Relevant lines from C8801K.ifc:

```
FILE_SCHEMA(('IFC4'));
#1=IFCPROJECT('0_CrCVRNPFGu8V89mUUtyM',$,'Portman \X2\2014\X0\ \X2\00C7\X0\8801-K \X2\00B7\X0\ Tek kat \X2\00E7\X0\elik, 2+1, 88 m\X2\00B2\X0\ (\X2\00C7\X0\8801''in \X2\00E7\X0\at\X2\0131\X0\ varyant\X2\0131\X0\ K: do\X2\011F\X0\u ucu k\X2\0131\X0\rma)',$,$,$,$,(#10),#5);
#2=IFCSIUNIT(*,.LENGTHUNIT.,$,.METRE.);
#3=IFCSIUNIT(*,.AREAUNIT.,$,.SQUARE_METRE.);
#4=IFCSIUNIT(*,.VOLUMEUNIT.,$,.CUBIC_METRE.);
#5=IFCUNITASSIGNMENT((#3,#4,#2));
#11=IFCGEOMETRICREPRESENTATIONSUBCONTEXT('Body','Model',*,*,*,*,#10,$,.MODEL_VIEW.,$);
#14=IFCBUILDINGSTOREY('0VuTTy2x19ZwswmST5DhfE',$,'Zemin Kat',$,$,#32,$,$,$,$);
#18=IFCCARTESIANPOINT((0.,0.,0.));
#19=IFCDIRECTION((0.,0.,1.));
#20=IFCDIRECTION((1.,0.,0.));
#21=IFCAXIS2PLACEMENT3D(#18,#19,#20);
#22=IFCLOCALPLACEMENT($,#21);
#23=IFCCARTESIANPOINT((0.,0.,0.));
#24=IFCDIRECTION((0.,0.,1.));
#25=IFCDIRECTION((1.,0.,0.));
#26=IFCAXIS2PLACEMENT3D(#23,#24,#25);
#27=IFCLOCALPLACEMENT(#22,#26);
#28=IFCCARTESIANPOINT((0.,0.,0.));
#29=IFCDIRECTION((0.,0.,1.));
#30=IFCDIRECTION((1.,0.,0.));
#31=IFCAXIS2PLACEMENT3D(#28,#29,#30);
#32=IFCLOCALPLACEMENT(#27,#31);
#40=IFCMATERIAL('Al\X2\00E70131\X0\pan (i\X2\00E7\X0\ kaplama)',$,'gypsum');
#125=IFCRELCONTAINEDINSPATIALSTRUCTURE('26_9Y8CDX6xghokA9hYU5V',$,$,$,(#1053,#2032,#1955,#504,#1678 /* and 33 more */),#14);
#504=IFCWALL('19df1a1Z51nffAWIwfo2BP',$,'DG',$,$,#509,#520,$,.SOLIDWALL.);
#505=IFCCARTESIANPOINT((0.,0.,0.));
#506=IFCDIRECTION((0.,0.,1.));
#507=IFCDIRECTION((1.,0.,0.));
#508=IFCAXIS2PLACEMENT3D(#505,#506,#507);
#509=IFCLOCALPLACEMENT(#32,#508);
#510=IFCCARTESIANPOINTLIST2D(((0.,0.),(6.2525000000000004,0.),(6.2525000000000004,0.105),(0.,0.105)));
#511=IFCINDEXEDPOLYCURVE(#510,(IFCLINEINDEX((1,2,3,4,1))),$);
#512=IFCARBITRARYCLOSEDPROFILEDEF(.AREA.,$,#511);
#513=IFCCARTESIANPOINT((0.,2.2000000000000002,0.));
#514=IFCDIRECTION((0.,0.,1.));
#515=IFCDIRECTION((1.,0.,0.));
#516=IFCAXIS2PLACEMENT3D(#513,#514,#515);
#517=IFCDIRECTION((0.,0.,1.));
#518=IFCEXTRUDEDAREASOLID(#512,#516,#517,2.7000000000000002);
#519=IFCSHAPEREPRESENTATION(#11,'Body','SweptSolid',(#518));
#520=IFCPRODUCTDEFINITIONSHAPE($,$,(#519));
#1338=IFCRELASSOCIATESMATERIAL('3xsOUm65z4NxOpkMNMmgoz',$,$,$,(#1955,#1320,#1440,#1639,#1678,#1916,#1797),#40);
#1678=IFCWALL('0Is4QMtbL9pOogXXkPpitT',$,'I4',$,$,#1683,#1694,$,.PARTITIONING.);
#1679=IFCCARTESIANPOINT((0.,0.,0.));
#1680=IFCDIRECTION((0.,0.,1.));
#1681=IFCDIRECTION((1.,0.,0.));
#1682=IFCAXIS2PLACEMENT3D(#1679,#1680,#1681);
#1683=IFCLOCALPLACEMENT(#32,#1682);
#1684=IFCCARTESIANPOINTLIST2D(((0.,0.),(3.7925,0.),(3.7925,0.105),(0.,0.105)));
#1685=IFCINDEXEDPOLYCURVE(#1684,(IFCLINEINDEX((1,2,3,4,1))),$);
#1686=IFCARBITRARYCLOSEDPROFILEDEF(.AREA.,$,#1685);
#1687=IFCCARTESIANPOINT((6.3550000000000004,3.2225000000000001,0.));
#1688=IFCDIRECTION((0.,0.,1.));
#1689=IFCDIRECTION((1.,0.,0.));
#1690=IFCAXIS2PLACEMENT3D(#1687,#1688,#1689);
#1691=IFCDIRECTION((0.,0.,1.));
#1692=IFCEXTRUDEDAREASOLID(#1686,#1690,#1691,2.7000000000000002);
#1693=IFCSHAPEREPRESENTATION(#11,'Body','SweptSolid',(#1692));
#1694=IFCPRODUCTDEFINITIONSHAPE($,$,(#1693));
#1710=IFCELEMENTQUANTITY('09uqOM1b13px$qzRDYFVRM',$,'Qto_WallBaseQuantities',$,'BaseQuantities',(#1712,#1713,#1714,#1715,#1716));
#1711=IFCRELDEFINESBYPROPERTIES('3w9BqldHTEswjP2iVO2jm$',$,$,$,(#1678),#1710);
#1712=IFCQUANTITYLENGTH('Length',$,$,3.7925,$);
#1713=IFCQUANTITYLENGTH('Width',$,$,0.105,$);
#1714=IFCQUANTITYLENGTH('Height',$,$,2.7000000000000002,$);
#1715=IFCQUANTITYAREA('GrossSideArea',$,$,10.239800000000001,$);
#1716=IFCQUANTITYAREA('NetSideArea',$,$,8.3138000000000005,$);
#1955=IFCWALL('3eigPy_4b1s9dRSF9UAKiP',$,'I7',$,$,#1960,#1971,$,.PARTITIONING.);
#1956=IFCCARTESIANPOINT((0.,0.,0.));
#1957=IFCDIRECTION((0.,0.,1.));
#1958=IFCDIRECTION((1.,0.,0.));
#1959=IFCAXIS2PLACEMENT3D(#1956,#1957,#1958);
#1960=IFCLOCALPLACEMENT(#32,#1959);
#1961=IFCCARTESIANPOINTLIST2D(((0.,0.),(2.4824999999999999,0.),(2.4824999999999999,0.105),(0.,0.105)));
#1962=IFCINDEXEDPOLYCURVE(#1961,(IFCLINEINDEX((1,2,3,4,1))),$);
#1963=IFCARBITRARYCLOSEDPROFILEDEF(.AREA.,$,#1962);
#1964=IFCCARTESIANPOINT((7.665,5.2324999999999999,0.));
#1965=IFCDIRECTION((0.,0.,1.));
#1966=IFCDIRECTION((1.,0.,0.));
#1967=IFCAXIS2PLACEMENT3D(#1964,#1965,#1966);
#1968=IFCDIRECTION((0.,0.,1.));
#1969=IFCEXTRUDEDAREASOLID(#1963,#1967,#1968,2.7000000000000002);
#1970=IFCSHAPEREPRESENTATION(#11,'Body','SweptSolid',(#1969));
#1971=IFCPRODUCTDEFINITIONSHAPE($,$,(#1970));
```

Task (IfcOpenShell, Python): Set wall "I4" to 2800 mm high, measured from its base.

```python
import ifcopenshell
import ifcopenshell.api.pset
import ifcopenshell.geom
import ifcopenshell.util.element
import ifcopenshell.util.representation
import ifcopenshell.util.shape
import ifcopenshell.util.unit

model = ifcopenshell.open("C8801K.ifc")
unit_scale = ifcopenshell.util.unit.calculate_unit_scale(model)
area_scale = ifcopenshell.util.unit.calculate_unit_scale(model, "AREAUNIT")
settings = ifcopenshell.geom.settings()


def volume(element):
    """Net volume in cubic metres, openings subtracted."""
    shape = ifcopenshell.geom.create_shape(settings, element)
    return ifcopenshell.util.shape.get_volume(shape.geometry)


wall = model.by_id(1678)
before = volume(wall)

body = ifcopenshell.util.representation.get_representation(wall, "Model", "Body")
solid = body.Items[0]
old_height = solid.Depth
solid.Depth = 2.8 / unit_scale
after = volume(wall)
thickness = 0.105  # wall thickness in metres

# Update the stored height, areas and volumes.
qto = model.by_id(ifcopenshell.util.element.get_pset(wall, "Qto_WallBaseQuantities", should_inherit=False)["id"])
ifcopenshell.api.pset.edit_qto(model, qto=qto, properties={
    "Height": solid.Depth,
    "GrossSideArea": ifcopenshell.util.element.get_pset(wall, "Qto_WallBaseQuantities", "GrossSideArea") * solid.Depth / old_height,
    "NetSideArea": after / thickness / area_scale,
})

print(f"height {old_height:g} -> {solid.Depth:g}, volume {before:.3f} -> {after:.3f} m3")

model.write("C8801K_rev.ifc")
```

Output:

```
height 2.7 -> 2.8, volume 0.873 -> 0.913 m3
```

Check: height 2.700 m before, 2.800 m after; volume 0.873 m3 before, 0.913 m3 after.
